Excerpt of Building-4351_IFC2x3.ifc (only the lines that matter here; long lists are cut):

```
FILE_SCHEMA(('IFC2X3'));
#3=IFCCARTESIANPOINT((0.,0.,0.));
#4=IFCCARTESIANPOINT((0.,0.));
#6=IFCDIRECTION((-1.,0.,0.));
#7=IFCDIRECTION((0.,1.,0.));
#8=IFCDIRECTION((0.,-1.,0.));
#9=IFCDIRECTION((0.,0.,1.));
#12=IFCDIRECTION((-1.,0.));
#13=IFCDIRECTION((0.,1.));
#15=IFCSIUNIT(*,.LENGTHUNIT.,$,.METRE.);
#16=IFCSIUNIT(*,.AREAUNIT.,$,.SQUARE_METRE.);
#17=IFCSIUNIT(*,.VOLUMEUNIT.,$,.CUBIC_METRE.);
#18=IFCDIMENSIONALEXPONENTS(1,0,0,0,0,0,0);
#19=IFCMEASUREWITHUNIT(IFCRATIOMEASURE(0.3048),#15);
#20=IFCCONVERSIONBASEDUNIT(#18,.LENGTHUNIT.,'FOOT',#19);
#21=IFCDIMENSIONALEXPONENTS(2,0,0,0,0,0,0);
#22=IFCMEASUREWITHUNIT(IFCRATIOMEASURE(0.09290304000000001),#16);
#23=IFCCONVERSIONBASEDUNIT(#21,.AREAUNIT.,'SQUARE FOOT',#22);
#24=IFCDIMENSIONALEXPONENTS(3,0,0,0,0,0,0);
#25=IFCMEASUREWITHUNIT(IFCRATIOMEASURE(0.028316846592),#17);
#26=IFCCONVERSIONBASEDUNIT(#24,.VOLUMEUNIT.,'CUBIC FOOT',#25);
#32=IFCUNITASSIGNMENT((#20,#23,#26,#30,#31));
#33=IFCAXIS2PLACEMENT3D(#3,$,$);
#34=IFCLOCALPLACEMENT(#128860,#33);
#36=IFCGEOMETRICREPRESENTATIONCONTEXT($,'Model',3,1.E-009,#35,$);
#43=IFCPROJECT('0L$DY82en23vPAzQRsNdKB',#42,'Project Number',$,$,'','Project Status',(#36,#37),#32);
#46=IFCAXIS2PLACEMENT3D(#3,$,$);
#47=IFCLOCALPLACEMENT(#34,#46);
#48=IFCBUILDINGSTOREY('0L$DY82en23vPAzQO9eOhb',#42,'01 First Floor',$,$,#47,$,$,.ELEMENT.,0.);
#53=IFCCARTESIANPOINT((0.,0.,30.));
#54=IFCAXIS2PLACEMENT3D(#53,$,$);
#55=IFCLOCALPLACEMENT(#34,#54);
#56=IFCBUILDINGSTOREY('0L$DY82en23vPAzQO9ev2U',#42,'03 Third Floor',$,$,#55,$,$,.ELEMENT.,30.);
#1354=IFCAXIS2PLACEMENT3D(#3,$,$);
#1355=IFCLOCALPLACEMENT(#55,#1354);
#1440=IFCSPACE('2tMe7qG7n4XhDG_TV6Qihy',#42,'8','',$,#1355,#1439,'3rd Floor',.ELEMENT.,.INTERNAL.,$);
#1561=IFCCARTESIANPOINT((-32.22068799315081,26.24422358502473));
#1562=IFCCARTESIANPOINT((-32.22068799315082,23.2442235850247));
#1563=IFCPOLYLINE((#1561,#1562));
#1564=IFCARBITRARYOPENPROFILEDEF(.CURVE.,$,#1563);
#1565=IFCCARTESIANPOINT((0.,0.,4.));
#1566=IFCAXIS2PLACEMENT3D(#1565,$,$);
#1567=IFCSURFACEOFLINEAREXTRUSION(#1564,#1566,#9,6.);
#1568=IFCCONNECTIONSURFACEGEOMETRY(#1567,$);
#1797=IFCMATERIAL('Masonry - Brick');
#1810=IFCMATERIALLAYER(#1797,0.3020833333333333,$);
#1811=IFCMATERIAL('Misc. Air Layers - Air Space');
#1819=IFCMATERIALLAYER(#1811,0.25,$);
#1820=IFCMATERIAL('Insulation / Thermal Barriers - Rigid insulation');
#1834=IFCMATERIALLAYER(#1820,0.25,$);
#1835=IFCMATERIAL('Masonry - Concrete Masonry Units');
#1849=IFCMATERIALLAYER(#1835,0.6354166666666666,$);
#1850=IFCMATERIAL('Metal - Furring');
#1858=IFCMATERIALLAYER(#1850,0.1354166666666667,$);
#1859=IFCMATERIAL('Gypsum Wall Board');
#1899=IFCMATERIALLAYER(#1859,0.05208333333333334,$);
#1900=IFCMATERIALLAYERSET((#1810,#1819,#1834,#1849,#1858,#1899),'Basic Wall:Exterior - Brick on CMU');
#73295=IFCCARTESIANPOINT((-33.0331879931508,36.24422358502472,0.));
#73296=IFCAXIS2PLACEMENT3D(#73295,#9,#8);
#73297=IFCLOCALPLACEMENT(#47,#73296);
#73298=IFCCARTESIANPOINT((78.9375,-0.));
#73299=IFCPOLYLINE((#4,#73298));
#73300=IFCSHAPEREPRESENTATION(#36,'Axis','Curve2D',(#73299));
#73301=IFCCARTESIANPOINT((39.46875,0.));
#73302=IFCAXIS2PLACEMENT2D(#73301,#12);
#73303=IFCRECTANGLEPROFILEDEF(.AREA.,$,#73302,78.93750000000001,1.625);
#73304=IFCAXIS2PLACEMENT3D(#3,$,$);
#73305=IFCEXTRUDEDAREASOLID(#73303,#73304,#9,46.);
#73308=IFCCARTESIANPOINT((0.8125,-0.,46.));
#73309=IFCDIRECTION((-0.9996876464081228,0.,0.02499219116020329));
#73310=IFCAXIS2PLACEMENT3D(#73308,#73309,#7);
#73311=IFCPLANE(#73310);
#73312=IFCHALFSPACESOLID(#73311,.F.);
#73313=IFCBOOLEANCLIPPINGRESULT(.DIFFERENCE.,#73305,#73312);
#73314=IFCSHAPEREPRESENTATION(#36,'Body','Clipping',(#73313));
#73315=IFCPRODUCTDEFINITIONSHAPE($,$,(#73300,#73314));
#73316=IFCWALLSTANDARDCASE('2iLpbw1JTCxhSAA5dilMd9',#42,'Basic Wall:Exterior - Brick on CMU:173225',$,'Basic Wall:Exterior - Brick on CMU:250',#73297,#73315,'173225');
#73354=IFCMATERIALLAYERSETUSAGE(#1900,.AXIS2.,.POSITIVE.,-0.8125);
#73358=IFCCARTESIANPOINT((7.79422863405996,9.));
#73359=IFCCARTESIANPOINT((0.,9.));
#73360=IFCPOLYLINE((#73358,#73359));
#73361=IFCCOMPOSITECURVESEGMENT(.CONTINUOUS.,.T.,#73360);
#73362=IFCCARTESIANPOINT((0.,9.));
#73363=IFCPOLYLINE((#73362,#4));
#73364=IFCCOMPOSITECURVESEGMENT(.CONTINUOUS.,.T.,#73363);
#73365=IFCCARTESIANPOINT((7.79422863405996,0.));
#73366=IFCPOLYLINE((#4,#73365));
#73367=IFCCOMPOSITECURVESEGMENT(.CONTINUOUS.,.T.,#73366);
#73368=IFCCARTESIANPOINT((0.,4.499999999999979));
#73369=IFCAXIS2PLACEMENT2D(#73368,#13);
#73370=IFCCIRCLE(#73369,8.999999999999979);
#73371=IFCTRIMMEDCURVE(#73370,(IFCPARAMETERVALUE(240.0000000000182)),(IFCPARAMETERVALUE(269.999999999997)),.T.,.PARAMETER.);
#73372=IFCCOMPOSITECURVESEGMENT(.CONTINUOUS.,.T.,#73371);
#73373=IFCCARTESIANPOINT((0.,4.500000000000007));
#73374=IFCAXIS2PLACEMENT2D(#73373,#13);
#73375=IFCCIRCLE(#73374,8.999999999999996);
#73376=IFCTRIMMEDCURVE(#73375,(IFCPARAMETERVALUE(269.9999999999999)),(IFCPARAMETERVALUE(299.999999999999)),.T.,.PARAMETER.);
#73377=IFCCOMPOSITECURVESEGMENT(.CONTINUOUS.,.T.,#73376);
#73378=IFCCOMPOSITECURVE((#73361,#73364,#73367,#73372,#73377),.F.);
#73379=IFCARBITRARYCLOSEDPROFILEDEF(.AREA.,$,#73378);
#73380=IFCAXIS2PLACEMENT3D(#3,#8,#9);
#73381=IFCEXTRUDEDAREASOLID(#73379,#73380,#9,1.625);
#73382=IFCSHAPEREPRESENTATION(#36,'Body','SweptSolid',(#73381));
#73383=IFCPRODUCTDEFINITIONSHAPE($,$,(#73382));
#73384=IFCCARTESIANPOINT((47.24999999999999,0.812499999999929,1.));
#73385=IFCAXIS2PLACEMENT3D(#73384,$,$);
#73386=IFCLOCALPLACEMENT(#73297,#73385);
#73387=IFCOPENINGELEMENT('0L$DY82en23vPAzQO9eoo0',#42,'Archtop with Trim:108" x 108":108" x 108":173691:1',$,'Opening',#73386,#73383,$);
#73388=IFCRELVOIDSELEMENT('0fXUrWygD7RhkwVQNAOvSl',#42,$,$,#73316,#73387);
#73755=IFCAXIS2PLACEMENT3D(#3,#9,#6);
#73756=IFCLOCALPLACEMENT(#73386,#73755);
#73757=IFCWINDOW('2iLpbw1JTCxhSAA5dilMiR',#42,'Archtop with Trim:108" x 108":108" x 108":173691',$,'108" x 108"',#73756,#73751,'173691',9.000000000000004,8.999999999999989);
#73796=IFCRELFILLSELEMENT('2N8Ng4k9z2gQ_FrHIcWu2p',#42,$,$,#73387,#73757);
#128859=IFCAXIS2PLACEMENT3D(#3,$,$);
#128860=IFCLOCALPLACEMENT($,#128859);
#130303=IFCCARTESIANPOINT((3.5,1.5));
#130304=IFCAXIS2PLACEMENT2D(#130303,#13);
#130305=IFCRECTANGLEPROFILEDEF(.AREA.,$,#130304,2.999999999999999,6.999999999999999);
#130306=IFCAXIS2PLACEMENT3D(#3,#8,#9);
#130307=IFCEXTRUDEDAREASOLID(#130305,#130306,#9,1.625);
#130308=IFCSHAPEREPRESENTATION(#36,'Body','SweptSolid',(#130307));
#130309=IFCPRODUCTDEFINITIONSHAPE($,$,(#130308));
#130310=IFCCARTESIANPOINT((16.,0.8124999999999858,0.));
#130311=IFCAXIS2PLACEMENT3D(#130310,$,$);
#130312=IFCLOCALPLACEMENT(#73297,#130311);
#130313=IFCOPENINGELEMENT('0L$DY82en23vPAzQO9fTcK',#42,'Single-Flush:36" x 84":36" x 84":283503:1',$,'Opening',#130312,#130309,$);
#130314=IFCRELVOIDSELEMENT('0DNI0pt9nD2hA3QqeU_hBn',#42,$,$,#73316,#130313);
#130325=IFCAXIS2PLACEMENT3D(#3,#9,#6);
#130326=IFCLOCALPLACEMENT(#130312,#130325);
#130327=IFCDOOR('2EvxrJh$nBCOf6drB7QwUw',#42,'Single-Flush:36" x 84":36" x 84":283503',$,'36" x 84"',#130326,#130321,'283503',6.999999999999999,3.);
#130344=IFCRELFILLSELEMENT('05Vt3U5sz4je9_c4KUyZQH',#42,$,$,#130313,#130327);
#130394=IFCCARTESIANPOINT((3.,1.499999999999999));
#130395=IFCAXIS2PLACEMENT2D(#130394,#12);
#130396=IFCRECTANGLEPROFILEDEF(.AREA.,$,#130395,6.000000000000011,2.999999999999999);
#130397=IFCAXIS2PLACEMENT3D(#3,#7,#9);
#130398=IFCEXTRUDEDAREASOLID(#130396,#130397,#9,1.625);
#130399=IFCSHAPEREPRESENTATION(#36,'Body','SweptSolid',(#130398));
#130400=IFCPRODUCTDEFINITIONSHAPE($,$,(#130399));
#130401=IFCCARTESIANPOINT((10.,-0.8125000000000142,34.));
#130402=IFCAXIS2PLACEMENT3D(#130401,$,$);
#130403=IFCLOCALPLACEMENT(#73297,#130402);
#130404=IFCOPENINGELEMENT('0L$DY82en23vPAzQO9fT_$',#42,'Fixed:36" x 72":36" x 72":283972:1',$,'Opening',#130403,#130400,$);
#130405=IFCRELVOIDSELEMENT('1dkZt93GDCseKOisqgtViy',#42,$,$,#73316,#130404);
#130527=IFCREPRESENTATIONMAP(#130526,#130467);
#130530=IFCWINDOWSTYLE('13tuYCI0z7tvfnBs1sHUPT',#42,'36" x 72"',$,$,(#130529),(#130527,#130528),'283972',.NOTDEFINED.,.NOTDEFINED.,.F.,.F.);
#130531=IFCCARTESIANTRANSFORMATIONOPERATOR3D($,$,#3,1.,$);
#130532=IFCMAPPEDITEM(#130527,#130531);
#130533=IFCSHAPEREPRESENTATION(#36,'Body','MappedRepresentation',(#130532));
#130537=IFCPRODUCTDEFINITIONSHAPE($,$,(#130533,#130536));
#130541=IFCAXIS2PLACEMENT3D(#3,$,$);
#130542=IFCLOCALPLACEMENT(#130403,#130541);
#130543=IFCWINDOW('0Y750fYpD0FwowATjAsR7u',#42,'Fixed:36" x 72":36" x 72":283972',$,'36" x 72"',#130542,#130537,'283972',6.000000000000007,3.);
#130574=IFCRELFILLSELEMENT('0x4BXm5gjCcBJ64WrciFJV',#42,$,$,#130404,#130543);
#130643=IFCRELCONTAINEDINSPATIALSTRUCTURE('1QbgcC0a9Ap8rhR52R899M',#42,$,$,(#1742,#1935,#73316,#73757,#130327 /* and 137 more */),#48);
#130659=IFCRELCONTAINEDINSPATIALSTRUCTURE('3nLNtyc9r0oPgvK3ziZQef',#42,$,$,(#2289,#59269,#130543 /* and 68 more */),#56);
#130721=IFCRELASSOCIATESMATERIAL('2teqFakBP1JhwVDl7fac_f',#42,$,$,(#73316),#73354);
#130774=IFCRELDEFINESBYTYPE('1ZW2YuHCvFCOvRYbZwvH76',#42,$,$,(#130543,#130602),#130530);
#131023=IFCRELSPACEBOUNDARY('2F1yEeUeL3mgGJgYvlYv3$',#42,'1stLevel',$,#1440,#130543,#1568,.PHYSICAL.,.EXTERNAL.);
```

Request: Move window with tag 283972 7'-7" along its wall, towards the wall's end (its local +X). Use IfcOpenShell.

```python
import numpy as np
import ifcopenshell
import ifcopenshell.api.geometry
import ifcopenshell.util.placement
import ifcopenshell.util.unit

model = ifcopenshell.open("Building-4351_IFC2x3.ifc")
unit_scale = ifcopenshell.util.unit.calculate_unit_scale(model)

window = model.by_id(130543)
opening = window.FillsVoids[0].RelatingOpeningElement
wall = opening.VoidsElements[0].RelatingBuildingElement

wall_matrix = ifcopenshell.util.placement.get_local_placement(wall.ObjectPlacement)
shift = wall_matrix[:3, 0] * 91 * 0.0254 / unit_scale
before = ifcopenshell.util.placement.get_local_placement(window.ObjectPlacement)[:3, 3].copy()

# The window is placed relative to its opening, so it follows when the opening moves.
matrix = ifcopenshell.util.placement.get_local_placement(opening.ObjectPlacement)
matrix[:3, 3] += shift
ifcopenshell.api.geometry.edit_object_placement(
    model, product=opening, matrix=matrix, is_si=False, should_transform_children=True
)

# Space boundary surfaces are stored in each space's coordinates; move them too.
for rel in window.ProvidesBoundaries:
    if not rel.ConnectionGeometry:
        continue
    surface = rel.ConnectionGeometry.SurfaceOnRelatingElement
    space_matrix = ifcopenshell.util.placement.get_local_placement(rel.RelatingSpace.ObjectPlacement)
    point = np.array(surface.Position.Location.Coordinates) + space_matrix[:3, :3].T @ shift
    surface.Position = model.createIfcAxis2Placement3D(
        model.createIfcCartesianPoint(point.tolist()), surface.Position.Axis, surface.Position.RefDirection
    )

after = ifcopenshell.util.placement.get_local_placement(window.ObjectPlacement)[:3, 3]
print("window moved by", (after - before).round(3) + 0.0)

model.write("Building-4351_IFC2x3_rev.ifc")
```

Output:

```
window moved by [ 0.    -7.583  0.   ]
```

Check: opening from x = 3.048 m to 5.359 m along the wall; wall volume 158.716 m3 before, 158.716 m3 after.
